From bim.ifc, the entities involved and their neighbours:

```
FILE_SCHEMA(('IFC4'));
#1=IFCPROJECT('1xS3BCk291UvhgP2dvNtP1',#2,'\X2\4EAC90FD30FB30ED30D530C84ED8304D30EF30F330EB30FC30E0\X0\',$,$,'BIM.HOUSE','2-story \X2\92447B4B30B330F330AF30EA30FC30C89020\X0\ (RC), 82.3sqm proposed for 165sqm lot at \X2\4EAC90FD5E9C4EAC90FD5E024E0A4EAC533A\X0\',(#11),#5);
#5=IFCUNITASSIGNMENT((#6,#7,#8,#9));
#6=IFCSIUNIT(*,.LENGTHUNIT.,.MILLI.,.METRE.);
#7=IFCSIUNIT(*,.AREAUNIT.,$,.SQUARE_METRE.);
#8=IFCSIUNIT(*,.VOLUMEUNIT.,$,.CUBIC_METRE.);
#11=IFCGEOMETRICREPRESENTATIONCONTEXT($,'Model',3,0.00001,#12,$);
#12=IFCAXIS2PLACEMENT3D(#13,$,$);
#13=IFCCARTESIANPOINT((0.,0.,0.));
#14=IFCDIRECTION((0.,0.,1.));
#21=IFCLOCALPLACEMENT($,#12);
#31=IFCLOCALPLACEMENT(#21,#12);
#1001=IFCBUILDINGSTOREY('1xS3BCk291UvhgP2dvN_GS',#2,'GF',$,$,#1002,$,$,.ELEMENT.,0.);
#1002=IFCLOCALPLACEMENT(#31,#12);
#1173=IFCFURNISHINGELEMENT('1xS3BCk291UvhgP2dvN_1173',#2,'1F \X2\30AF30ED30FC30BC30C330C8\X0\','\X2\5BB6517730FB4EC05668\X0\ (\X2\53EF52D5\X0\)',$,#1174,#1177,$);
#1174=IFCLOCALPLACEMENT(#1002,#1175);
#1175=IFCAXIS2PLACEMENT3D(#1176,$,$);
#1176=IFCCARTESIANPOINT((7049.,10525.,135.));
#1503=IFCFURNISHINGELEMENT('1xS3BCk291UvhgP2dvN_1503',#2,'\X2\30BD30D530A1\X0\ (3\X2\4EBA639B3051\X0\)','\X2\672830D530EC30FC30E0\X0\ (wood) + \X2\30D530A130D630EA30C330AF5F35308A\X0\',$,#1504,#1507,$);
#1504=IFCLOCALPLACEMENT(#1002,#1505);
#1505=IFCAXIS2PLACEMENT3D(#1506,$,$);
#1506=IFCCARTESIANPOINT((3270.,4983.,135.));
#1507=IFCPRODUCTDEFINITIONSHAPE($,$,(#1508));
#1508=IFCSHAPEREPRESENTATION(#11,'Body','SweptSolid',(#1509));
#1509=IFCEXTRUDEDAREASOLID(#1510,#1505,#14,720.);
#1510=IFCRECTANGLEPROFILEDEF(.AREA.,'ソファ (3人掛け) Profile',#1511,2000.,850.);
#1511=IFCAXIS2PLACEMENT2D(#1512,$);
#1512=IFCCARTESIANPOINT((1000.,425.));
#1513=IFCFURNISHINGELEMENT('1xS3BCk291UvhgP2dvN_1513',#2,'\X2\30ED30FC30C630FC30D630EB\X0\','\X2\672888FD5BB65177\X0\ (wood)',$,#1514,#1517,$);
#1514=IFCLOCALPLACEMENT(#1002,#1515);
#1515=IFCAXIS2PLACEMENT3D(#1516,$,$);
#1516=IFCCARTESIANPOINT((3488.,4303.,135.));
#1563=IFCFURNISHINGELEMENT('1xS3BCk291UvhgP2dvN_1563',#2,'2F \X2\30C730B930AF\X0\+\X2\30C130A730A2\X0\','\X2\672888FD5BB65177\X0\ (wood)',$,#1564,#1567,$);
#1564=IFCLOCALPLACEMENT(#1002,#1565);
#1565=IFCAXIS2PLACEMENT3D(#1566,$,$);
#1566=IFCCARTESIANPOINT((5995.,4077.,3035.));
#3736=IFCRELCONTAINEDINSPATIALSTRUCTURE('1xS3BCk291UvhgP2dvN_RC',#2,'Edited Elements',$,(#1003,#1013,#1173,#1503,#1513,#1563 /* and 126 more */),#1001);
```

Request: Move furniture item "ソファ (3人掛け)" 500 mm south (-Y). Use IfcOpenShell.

```python
import ifcopenshell
import ifcopenshell.api.geometry
import ifcopenshell.util.placement
import ifcopenshell.util.unit

model = ifcopenshell.open("bim.ifc")
unit_scale = ifcopenshell.util.unit.calculate_unit_scale(model)

item = model.by_guid("1xS3BCk291UvhgP2dvN_1503")
matrix = ifcopenshell.util.placement.get_local_placement(item.ObjectPlacement)
matrix[1, 3] -= 0.5 / unit_scale
ifcopenshell.api.geometry.edit_object_placement(model, product=item, matrix=matrix, is_si=False)

print(ifcopenshell.util.placement.get_local_placement(item.ObjectPlacement).round(3) + 0.0)

model.write("bim_updated.ifc")
```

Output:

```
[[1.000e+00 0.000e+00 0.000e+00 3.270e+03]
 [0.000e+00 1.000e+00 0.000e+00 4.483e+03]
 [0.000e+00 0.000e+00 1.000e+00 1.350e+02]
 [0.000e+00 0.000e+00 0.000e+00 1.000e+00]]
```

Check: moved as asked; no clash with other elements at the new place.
